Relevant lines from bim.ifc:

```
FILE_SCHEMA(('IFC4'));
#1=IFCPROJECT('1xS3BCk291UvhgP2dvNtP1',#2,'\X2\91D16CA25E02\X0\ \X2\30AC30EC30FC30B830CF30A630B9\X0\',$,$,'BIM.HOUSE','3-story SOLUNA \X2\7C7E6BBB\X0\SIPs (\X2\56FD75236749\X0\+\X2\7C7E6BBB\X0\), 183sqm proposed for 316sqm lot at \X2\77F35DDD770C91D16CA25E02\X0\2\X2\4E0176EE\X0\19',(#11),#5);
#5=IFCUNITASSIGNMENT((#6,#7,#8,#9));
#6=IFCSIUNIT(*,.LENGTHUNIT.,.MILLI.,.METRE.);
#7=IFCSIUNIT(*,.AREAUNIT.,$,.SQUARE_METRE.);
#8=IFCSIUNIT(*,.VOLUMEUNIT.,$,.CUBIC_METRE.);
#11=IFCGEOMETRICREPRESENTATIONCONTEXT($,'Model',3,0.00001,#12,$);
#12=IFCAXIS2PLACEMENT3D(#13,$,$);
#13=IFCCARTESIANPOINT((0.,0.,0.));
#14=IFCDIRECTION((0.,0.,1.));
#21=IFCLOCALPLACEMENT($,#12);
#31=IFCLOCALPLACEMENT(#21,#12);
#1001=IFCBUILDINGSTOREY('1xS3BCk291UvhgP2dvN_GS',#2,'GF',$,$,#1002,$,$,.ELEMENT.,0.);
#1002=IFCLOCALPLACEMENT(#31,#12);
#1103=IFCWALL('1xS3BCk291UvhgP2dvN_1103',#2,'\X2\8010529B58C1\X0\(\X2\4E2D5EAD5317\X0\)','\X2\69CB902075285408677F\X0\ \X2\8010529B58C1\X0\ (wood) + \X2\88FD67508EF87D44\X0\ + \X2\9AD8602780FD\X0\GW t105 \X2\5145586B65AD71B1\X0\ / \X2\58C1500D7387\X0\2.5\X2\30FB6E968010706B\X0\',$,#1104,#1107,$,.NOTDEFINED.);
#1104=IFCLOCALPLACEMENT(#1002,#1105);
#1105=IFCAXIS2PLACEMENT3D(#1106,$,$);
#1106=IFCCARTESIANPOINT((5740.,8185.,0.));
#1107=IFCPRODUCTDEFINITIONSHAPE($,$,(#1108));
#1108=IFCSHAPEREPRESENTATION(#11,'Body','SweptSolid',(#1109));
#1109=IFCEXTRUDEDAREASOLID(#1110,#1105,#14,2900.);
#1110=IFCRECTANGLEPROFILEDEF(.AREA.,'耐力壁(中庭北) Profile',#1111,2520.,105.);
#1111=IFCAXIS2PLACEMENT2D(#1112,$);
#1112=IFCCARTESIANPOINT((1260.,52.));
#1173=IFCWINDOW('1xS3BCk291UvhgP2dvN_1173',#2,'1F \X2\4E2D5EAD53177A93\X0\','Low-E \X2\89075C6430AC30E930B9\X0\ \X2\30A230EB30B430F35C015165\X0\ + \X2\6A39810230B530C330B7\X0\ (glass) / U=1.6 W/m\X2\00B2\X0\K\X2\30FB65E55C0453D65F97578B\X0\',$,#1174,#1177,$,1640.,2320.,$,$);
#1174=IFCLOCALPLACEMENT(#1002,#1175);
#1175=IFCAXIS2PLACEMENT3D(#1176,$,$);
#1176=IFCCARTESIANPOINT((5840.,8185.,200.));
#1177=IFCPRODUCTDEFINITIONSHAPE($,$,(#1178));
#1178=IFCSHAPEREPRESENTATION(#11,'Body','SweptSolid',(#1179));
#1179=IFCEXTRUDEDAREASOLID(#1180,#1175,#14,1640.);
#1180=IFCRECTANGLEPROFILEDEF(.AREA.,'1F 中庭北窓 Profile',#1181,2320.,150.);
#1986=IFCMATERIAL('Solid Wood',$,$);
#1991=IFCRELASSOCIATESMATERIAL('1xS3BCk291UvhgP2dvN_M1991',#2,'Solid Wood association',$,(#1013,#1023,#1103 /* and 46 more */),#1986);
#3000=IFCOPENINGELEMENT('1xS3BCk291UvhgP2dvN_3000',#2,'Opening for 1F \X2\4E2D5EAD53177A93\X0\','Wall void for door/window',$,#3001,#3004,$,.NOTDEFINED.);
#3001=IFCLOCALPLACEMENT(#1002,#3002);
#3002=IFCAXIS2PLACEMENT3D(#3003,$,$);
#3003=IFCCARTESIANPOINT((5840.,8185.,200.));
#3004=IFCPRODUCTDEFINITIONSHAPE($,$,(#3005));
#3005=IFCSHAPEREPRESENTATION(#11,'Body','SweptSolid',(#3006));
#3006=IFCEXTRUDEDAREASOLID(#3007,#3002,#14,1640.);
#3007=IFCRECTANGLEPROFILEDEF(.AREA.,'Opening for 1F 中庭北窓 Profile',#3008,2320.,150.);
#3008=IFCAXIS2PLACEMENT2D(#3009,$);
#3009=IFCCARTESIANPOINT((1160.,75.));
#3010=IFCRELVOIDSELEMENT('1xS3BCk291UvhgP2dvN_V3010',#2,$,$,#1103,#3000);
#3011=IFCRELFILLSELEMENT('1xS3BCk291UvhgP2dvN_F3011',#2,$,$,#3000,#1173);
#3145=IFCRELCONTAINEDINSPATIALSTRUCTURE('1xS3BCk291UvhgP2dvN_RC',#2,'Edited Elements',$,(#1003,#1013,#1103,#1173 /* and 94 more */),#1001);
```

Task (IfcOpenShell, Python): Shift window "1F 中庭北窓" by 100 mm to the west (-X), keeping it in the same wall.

```python
import ifcopenshell
import ifcopenshell.api.geometry
import ifcopenshell.util.placement

model = ifcopenshell.open("bim.ifc")

window = model.by_guid("1xS3BCk291UvhgP2dvN_1173")
opening = window.FillsVoids[0].RelatingOpeningElement
wall = opening.VoidsElements[0].RelatingBuildingElement

wall_matrix = ifcopenshell.util.placement.get_local_placement(wall.ObjectPlacement)
shift = wall_matrix[:3, 0] * -100.0
before = ifcopenshell.util.placement.get_local_placement(window.ObjectPlacement)[:3, 3].copy()

# The window is not placed relative to its opening, so move both.
for product in (opening, window):
    matrix = ifcopenshell.util.placement.get_local_placement(product.ObjectPlacement)
    matrix[:3, 3] += shift
    ifcopenshell.api.geometry.edit_object_placement(model, product=product, matrix=matrix, is_si=False)

after = ifcopenshell.util.placement.get_local_placement(window.ObjectPlacement)[:3, 3]
print("window moved by", (after - before).round(3) + 0.0)

model.write("bim-out.ifc")
```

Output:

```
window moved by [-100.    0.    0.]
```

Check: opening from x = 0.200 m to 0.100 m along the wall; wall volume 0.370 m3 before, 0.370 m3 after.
